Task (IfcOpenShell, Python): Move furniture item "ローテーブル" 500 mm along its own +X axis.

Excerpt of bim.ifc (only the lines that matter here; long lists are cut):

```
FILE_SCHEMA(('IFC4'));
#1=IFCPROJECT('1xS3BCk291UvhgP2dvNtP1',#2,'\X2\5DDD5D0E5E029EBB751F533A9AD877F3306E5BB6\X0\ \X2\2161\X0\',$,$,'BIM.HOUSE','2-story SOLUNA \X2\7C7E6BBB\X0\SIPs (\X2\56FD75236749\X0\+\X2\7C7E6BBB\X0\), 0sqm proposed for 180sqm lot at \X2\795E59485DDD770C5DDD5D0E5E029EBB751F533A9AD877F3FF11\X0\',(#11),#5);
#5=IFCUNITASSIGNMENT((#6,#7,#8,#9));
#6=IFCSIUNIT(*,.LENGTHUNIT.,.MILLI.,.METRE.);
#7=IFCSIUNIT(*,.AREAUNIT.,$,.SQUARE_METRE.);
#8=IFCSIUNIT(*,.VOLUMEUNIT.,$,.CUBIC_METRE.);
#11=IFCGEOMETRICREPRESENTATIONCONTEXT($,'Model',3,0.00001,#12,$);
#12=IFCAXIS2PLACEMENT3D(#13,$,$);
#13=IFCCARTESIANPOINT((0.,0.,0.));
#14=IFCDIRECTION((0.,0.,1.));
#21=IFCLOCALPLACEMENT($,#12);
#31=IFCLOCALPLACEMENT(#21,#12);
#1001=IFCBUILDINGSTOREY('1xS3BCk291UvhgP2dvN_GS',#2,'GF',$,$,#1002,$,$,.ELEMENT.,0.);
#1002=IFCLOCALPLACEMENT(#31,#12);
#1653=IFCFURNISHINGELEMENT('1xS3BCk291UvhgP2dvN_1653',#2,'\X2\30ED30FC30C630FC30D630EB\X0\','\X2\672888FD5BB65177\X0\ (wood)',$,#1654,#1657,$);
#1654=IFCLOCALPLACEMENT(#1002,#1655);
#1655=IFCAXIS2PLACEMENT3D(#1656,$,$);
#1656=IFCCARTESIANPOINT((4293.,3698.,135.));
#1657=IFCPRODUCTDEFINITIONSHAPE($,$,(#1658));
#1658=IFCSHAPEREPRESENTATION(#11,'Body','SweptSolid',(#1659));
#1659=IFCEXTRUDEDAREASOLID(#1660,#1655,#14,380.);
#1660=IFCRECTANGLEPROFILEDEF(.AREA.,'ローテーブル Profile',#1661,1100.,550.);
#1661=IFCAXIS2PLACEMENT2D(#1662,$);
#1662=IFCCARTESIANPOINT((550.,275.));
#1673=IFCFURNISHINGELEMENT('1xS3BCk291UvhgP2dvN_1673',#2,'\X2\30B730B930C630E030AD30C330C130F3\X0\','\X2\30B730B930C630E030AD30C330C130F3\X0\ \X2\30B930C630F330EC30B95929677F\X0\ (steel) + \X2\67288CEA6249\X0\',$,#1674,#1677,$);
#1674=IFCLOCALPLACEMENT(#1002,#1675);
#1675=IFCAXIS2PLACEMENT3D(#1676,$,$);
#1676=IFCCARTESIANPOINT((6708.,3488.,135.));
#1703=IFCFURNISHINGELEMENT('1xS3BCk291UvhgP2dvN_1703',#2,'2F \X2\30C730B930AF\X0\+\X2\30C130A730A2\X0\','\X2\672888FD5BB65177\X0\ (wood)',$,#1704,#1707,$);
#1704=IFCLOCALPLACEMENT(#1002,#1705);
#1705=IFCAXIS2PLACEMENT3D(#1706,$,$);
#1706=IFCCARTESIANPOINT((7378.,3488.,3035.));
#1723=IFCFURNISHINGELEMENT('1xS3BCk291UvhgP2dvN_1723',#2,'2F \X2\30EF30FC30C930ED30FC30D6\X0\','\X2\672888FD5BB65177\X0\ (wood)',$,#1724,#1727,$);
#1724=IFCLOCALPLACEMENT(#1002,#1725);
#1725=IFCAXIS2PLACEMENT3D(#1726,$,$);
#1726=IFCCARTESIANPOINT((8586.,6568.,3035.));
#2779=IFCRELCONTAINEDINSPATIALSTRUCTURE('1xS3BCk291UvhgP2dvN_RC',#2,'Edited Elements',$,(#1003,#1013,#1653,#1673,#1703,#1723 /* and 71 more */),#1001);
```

```python
import ifcopenshell
import ifcopenshell.api.geometry
import ifcopenshell.util.placement
import ifcopenshell.util.unit

model = ifcopenshell.open("bim.ifc")
unit_scale = ifcopenshell.util.unit.calculate_unit_scale(model)

item = model.by_guid("1xS3BCk291UvhgP2dvN_1653")
matrix = ifcopenshell.util.placement.get_local_placement(item.ObjectPlacement)
matrix[:3, 3] += matrix[:3, 0] * 0.5 / unit_scale
ifcopenshell.api.geometry.edit_object_placement(model, product=item, matrix=matrix, is_si=False)

print(ifcopenshell.util.placement.get_local_placement(item.ObjectPlacement).round(3) + 0.0)

model.write("bim_rev.ifc")
```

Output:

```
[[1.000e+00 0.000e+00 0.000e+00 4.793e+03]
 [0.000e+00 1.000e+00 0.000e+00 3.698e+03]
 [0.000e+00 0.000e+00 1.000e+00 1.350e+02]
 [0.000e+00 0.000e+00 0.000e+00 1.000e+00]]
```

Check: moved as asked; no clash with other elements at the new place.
